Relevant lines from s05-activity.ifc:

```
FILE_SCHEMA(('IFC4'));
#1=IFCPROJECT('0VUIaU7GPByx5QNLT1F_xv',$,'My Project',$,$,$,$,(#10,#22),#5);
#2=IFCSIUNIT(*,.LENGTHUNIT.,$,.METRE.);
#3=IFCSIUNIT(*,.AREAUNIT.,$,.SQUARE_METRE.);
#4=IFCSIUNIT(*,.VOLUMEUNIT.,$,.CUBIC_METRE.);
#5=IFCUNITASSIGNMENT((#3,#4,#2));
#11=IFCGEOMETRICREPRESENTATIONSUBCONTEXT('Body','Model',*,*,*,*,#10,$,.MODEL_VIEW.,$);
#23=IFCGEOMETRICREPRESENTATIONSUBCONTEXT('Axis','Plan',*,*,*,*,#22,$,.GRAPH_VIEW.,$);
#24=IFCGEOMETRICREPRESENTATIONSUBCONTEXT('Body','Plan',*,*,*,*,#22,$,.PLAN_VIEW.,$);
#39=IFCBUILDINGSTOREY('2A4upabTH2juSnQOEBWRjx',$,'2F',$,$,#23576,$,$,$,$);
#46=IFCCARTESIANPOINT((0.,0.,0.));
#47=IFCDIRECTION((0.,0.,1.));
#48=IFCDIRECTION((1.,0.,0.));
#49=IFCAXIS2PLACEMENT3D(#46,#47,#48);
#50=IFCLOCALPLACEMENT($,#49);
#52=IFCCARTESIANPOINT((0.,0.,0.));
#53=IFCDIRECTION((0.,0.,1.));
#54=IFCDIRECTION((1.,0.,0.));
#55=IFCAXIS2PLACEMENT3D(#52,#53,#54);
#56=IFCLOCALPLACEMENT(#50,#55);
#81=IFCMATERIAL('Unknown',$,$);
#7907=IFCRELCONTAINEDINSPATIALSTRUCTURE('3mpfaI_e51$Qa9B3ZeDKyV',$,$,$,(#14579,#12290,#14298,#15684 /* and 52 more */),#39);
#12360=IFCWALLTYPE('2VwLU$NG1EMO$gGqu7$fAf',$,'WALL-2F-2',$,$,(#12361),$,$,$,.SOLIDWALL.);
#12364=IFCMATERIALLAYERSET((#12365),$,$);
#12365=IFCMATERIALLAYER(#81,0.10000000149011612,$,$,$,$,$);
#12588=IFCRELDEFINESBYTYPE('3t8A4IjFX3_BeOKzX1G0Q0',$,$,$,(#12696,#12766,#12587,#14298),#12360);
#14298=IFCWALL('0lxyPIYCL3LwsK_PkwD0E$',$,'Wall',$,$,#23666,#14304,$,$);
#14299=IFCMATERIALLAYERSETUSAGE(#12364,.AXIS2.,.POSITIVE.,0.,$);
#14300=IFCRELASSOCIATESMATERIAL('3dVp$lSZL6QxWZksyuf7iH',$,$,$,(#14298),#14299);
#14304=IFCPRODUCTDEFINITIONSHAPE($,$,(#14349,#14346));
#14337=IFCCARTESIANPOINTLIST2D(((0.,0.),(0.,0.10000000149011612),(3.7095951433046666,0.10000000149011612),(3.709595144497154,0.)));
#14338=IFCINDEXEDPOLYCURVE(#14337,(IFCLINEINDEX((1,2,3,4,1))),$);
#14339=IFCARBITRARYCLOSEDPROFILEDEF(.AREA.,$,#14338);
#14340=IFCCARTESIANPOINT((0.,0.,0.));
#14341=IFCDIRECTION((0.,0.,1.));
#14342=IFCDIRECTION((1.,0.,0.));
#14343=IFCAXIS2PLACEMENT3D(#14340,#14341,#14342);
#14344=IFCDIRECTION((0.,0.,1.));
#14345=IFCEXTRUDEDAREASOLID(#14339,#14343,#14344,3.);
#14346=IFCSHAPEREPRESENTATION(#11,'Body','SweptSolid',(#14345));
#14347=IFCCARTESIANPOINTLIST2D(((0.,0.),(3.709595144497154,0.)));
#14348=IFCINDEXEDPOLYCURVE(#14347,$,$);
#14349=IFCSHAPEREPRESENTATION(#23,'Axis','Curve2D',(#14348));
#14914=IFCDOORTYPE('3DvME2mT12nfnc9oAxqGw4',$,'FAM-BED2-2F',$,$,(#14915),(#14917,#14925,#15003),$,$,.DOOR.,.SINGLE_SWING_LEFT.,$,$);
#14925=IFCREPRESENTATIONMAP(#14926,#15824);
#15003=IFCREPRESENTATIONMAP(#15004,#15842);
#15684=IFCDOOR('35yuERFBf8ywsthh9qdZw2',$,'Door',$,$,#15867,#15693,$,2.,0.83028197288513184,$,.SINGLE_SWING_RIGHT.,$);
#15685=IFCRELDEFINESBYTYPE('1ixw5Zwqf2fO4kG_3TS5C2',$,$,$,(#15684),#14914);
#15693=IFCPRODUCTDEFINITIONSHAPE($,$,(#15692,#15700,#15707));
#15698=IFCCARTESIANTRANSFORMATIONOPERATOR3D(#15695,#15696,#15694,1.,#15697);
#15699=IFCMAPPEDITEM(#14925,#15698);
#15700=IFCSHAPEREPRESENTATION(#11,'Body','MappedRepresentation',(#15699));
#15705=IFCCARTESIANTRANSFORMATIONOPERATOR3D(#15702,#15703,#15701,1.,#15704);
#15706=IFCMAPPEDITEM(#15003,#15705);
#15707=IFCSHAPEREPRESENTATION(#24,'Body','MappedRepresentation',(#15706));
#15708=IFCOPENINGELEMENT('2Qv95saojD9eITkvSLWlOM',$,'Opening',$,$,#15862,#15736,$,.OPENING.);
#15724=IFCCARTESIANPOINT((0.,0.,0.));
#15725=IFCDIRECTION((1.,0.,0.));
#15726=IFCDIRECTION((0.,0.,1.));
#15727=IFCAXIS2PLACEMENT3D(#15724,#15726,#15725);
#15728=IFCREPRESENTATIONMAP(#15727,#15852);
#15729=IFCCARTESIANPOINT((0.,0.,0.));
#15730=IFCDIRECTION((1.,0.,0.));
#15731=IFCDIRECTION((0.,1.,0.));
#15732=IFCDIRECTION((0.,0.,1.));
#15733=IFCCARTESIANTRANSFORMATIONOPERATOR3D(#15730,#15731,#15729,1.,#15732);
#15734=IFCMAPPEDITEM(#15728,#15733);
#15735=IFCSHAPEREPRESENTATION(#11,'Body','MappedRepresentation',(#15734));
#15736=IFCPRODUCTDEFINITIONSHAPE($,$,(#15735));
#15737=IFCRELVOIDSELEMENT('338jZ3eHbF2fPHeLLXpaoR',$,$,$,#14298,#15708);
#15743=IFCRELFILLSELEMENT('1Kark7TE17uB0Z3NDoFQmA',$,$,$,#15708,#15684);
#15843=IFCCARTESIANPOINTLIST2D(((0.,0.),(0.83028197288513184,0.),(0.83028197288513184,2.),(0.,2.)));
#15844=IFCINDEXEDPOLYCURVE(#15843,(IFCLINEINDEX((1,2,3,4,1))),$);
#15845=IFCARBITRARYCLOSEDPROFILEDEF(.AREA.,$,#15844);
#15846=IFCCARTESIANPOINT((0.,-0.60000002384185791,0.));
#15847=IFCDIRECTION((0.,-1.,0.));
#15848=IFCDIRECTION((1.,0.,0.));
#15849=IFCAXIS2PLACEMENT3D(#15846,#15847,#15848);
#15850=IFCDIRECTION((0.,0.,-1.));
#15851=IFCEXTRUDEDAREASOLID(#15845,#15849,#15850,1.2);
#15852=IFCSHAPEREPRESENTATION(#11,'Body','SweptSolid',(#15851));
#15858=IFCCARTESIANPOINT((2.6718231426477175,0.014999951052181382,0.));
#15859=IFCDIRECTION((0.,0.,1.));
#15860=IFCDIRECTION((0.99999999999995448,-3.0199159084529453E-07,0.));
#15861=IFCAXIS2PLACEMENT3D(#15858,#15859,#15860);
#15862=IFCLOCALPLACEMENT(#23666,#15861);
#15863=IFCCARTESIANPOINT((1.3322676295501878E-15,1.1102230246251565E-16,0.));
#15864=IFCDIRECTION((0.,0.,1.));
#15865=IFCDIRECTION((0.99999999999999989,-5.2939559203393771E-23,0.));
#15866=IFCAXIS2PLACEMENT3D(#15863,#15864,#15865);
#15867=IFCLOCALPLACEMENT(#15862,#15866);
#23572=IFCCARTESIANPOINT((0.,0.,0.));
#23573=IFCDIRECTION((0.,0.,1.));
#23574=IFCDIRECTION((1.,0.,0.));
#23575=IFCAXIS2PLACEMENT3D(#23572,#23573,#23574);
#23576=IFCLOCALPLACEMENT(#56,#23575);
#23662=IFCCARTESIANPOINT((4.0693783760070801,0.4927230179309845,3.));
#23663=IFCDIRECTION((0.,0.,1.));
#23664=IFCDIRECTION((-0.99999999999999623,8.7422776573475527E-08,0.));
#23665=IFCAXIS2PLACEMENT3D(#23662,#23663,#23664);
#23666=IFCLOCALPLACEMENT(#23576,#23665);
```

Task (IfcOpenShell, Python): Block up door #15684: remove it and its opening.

```python
import ifcopenshell
import ifcopenshell.api.feature
import ifcopenshell.api.root
import ifcopenshell.geom
import ifcopenshell.util.shape

model = ifcopenshell.open("s05-activity.ifc")
settings = ifcopenshell.geom.settings()


def volume(element):
    """Net volume in cubic metres, openings subtracted."""
    shape = ifcopenshell.geom.create_shape(settings, element)
    return ifcopenshell.util.shape.get_volume(shape.geometry)


door = model.by_guid("35yuERFBf8ywsthh9qdZw2")
opening = door.FillsVoids[0].RelatingOpeningElement
wall = opening.VoidsElements[0].RelatingBuildingElement
before = volume(wall)

ifcopenshell.api.root.remove_product(model, product=door)
ifcopenshell.api.feature.remove_feature(model, feature=opening)

after = volume(wall)

print(f"wall volume {before:.3f} -> {after:.3f} m3")

model.write("s05-activity-out.ifc")
```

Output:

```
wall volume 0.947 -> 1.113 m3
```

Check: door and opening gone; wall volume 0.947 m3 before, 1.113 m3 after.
